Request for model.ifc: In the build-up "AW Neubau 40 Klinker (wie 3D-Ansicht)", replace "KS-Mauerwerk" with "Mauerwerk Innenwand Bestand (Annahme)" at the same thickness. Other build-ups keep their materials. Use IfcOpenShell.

First a look at what the model holds.

```python
import ifcopenshell
import ifcopenshell.util.element

model = ifcopenshell.open("model.ifc")
print(model.schema)
for layer_set in model.by_type("IfcMaterialLayerSet"):
    if layer_set.LayerSetName == "AW Neubau 40 Klinker (wie 3D-Ansicht)":
        for layer in layer_set.MaterialLayers:
            print(layer.id(), layer.Material and layer.Material.Name, layer.LayerThickness, sep=" | ")
        print(len(ifcopenshell.util.element.get_elements_by_material(model, layer_set)), "elements and types use it")
print(sorted(m.Name for m in model.by_type("IfcMaterial") if m.Name)[:60])
```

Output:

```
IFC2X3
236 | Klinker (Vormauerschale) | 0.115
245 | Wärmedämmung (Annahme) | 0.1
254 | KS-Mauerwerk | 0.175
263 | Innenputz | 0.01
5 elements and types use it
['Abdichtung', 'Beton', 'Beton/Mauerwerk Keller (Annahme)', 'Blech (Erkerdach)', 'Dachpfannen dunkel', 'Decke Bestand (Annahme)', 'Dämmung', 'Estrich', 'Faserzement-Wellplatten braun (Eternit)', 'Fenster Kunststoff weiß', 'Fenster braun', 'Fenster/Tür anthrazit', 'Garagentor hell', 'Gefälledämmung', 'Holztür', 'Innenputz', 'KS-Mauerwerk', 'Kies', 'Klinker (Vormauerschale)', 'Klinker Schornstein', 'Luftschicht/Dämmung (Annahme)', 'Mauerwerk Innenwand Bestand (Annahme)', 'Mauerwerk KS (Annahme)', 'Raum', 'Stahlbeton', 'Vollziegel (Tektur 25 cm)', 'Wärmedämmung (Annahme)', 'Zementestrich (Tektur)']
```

```python
import ifcopenshell
import ifcopenshell.api.material

model = ifcopenshell.open("model.ifc")

layer_set = next(s for s in model.by_type("IfcMaterialLayerSet") if s.LayerSetName == "AW Neubau 40 Klinker (wie 3D-Ansicht)")
layer = next(l for l in layer_set.MaterialLayers if l.Material and l.Material.Name == "KS-Mauerwerk")
material = next(m for m in model.by_type("IfcMaterial") if m.Name == "Mauerwerk Innenwand Bestand (Annahme)")

# Point this one layer at the other material; renaming the old one would change it everywhere.
ifcopenshell.api.material.edit_layer(model, layer=layer, attributes={}, material=material)

print([l.Material.Name if l.Material else None for l in layer_set.MaterialLayers])

model.write("model-out.ifc")
```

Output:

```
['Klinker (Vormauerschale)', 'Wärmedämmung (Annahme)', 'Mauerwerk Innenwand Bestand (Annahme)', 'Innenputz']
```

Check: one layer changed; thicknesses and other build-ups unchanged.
